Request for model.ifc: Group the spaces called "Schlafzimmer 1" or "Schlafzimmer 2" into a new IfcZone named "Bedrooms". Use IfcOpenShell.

First a look at what the model holds.

```python
import ifcopenshell

model = ifcopenshell.open("model.ifc")
print(model.schema)
seen = {}
for space in model.by_type("IfcSpace"):
    seen[space.LongName] = seen.get(space.LongName, 0) + 1
for name, count in sorted(seen.items(), key=str):
    print(count, "x", name)
print("zones:", [z.Name for z in model.by_type("IfcZone")][:20])
```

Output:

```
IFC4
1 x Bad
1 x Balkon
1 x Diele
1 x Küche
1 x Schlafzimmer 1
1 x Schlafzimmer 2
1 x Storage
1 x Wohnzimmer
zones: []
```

```python
import ifcopenshell
import ifcopenshell.api.group
import ifcopenshell.api.root

model = ifcopenshell.open("model.ifc")

names = {"Schlafzimmer 1", "Schlafzimmer 2"}
spaces = [s for s in model.by_type("IfcSpace") if s.LongName in names]

zone = ifcopenshell.api.root.create_entity(model, ifc_class="IfcZone", name="Bedrooms")
ifcopenshell.api.group.assign_group(model, products=spaces, group=zone)
print(len(spaces), "spaces in", zone.Name)

model.write("model_rev.ifc")
```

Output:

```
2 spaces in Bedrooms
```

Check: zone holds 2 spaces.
